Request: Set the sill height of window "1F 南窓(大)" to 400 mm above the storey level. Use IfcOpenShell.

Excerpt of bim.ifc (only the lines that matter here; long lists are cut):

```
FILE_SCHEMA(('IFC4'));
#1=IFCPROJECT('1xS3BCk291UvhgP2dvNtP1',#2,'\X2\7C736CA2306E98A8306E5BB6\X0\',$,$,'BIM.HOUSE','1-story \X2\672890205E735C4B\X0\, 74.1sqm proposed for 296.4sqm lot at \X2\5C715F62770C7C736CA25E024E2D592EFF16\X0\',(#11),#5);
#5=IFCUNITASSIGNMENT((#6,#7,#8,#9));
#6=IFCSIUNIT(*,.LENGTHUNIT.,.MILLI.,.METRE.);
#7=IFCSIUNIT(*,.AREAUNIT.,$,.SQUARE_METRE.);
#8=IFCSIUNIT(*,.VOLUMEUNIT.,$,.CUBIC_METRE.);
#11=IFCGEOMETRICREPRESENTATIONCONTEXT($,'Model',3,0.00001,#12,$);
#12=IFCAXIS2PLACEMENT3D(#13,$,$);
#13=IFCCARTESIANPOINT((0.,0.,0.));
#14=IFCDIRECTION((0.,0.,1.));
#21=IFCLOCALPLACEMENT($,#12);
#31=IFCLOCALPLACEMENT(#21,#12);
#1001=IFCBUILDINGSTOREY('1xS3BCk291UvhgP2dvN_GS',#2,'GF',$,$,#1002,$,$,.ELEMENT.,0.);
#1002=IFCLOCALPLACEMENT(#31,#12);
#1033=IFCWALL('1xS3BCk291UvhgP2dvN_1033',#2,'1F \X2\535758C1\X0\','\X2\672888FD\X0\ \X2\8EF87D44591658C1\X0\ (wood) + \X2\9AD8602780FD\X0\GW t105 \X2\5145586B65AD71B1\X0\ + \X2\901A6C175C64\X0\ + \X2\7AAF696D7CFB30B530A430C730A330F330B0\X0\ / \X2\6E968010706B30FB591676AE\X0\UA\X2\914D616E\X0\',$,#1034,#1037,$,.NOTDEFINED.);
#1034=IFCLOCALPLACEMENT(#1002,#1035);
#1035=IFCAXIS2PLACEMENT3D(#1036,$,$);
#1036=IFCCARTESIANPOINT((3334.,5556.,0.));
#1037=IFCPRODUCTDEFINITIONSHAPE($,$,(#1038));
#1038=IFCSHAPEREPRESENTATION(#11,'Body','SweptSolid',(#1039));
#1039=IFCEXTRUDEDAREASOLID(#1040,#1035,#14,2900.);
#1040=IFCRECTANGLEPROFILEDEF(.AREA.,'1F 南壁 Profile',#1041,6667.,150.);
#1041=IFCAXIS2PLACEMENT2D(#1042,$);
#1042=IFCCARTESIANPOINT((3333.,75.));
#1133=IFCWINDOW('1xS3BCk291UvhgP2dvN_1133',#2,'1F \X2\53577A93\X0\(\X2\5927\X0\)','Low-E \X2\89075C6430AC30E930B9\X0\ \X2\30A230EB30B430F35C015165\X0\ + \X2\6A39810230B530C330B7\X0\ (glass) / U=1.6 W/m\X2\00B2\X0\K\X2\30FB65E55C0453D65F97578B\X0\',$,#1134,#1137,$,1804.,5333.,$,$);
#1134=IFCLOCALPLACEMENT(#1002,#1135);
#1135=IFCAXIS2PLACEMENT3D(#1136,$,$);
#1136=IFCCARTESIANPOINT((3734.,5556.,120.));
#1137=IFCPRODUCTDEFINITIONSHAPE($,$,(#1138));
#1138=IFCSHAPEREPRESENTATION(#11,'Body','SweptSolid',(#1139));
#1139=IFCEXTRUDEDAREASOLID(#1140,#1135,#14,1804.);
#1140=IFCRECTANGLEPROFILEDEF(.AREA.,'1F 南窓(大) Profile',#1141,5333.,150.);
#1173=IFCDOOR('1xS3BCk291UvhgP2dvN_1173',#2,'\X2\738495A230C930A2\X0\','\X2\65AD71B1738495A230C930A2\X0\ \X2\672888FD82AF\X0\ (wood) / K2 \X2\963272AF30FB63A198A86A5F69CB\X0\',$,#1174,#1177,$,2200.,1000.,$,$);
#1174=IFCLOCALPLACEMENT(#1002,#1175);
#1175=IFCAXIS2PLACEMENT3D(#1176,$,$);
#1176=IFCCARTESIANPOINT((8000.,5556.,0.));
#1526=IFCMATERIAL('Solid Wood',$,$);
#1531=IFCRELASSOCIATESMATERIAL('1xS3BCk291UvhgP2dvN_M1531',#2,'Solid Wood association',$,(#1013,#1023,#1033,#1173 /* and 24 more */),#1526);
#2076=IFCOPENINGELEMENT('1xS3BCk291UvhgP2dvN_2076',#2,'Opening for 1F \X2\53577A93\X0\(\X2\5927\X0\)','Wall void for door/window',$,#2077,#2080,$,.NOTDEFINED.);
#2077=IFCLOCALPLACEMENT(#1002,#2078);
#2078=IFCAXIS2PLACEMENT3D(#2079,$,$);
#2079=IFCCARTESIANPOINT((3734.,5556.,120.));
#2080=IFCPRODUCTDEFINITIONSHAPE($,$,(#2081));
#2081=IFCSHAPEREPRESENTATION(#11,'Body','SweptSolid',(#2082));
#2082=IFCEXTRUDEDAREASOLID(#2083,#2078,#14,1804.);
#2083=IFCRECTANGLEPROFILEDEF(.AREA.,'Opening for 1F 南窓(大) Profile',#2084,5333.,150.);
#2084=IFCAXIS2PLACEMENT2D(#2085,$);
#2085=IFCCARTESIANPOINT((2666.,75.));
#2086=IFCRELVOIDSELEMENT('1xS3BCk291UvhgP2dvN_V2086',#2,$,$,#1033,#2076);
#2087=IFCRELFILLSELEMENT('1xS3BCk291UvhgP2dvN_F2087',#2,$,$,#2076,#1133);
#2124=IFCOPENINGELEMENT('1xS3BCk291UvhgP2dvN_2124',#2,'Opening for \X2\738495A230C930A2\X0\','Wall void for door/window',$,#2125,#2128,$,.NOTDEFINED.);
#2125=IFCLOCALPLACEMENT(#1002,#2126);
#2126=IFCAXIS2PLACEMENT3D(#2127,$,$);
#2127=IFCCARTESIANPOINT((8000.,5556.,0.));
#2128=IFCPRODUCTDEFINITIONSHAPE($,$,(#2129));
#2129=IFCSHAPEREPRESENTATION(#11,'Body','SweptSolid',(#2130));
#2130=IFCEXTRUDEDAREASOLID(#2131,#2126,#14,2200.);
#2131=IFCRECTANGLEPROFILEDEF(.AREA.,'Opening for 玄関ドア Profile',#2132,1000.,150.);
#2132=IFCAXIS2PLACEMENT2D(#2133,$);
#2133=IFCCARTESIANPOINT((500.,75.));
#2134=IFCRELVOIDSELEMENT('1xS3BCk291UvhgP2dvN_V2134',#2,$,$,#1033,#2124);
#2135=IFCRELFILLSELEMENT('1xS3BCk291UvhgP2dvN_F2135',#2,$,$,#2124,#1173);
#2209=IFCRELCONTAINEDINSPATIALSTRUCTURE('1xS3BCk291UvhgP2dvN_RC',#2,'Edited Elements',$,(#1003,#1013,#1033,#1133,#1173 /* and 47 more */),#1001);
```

```python
import numpy as np
import ifcopenshell
import ifcopenshell.api.geometry
import ifcopenshell.geom
import ifcopenshell.util.element
import ifcopenshell.util.placement
import ifcopenshell.util.shape
import ifcopenshell.util.unit

model = ifcopenshell.open("bim.ifc")
unit_scale = ifcopenshell.util.unit.calculate_unit_scale(model)

window = model.by_id(1133)
opening = window.FillsVoids[0].RelatingOpeningElement
storey = ifcopenshell.util.element.get_container(window, ifc_class="IfcBuildingStorey")
level = ifcopenshell.util.placement.get_local_placement(storey.ObjectPlacement)[2, 3]

# The opening's origin need not be at the sill, so measure its lowest point.
shape = ifcopenshell.geom.create_shape(ifcopenshell.geom.settings(), opening)
bottom = ifcopenshell.util.shape.get_shape_bottom_elevation(shape, shape.geometry) / unit_scale
dz = level + 400.0 - bottom

shift = np.array([0.0, 0.0, dz])
# The window is not placed relative to its opening, so move both.
for product in (opening, window):
    matrix = ifcopenshell.util.placement.get_local_placement(product.ObjectPlacement)
    matrix[:3, 3] += shift
    ifcopenshell.api.geometry.edit_object_placement(model, product=product, matrix=matrix, is_si=False)

print(f"moved by {dz * unit_scale:+.3f} m")

model.write("bim-out.ifc")
```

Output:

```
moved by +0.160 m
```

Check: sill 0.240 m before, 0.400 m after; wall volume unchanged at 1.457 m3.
